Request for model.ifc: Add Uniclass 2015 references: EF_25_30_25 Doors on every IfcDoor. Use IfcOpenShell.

First a look at what the model holds.

```python
import ifcopenshell

model = ifcopenshell.open("model.ifc")
print(model.schema)
print("classifications:", [c.Name for c in model.by_type("IfcClassification")])
for ifc_class in ("IfcDoor", "IfcRoof", "IfcStair", "IfcWall", "IfcWindow"):
    print(ifc_class, len(model.by_type(ifc_class)))
```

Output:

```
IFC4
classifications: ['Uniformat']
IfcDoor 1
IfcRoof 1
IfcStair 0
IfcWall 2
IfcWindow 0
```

```python
import ifcopenshell
import ifcopenshell.api.classification

model = ifcopenshell.open("model.ifc")

system = ifcopenshell.api.classification.add_classification(model, classification="Uniclass 2015")

codes = {
    "IfcDoor": ("EF_25_30_25", "Doors"),
}
for ifc_class, (code, name) in codes.items():
    products = model.by_type(ifc_class)
    ifcopenshell.api.classification.add_reference(
        model, products=products, classification=system, identification=code, name=name
    )
    print(code, len(products))

model.write("model_updated.ifc")
```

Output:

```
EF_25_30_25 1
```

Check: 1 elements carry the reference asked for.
